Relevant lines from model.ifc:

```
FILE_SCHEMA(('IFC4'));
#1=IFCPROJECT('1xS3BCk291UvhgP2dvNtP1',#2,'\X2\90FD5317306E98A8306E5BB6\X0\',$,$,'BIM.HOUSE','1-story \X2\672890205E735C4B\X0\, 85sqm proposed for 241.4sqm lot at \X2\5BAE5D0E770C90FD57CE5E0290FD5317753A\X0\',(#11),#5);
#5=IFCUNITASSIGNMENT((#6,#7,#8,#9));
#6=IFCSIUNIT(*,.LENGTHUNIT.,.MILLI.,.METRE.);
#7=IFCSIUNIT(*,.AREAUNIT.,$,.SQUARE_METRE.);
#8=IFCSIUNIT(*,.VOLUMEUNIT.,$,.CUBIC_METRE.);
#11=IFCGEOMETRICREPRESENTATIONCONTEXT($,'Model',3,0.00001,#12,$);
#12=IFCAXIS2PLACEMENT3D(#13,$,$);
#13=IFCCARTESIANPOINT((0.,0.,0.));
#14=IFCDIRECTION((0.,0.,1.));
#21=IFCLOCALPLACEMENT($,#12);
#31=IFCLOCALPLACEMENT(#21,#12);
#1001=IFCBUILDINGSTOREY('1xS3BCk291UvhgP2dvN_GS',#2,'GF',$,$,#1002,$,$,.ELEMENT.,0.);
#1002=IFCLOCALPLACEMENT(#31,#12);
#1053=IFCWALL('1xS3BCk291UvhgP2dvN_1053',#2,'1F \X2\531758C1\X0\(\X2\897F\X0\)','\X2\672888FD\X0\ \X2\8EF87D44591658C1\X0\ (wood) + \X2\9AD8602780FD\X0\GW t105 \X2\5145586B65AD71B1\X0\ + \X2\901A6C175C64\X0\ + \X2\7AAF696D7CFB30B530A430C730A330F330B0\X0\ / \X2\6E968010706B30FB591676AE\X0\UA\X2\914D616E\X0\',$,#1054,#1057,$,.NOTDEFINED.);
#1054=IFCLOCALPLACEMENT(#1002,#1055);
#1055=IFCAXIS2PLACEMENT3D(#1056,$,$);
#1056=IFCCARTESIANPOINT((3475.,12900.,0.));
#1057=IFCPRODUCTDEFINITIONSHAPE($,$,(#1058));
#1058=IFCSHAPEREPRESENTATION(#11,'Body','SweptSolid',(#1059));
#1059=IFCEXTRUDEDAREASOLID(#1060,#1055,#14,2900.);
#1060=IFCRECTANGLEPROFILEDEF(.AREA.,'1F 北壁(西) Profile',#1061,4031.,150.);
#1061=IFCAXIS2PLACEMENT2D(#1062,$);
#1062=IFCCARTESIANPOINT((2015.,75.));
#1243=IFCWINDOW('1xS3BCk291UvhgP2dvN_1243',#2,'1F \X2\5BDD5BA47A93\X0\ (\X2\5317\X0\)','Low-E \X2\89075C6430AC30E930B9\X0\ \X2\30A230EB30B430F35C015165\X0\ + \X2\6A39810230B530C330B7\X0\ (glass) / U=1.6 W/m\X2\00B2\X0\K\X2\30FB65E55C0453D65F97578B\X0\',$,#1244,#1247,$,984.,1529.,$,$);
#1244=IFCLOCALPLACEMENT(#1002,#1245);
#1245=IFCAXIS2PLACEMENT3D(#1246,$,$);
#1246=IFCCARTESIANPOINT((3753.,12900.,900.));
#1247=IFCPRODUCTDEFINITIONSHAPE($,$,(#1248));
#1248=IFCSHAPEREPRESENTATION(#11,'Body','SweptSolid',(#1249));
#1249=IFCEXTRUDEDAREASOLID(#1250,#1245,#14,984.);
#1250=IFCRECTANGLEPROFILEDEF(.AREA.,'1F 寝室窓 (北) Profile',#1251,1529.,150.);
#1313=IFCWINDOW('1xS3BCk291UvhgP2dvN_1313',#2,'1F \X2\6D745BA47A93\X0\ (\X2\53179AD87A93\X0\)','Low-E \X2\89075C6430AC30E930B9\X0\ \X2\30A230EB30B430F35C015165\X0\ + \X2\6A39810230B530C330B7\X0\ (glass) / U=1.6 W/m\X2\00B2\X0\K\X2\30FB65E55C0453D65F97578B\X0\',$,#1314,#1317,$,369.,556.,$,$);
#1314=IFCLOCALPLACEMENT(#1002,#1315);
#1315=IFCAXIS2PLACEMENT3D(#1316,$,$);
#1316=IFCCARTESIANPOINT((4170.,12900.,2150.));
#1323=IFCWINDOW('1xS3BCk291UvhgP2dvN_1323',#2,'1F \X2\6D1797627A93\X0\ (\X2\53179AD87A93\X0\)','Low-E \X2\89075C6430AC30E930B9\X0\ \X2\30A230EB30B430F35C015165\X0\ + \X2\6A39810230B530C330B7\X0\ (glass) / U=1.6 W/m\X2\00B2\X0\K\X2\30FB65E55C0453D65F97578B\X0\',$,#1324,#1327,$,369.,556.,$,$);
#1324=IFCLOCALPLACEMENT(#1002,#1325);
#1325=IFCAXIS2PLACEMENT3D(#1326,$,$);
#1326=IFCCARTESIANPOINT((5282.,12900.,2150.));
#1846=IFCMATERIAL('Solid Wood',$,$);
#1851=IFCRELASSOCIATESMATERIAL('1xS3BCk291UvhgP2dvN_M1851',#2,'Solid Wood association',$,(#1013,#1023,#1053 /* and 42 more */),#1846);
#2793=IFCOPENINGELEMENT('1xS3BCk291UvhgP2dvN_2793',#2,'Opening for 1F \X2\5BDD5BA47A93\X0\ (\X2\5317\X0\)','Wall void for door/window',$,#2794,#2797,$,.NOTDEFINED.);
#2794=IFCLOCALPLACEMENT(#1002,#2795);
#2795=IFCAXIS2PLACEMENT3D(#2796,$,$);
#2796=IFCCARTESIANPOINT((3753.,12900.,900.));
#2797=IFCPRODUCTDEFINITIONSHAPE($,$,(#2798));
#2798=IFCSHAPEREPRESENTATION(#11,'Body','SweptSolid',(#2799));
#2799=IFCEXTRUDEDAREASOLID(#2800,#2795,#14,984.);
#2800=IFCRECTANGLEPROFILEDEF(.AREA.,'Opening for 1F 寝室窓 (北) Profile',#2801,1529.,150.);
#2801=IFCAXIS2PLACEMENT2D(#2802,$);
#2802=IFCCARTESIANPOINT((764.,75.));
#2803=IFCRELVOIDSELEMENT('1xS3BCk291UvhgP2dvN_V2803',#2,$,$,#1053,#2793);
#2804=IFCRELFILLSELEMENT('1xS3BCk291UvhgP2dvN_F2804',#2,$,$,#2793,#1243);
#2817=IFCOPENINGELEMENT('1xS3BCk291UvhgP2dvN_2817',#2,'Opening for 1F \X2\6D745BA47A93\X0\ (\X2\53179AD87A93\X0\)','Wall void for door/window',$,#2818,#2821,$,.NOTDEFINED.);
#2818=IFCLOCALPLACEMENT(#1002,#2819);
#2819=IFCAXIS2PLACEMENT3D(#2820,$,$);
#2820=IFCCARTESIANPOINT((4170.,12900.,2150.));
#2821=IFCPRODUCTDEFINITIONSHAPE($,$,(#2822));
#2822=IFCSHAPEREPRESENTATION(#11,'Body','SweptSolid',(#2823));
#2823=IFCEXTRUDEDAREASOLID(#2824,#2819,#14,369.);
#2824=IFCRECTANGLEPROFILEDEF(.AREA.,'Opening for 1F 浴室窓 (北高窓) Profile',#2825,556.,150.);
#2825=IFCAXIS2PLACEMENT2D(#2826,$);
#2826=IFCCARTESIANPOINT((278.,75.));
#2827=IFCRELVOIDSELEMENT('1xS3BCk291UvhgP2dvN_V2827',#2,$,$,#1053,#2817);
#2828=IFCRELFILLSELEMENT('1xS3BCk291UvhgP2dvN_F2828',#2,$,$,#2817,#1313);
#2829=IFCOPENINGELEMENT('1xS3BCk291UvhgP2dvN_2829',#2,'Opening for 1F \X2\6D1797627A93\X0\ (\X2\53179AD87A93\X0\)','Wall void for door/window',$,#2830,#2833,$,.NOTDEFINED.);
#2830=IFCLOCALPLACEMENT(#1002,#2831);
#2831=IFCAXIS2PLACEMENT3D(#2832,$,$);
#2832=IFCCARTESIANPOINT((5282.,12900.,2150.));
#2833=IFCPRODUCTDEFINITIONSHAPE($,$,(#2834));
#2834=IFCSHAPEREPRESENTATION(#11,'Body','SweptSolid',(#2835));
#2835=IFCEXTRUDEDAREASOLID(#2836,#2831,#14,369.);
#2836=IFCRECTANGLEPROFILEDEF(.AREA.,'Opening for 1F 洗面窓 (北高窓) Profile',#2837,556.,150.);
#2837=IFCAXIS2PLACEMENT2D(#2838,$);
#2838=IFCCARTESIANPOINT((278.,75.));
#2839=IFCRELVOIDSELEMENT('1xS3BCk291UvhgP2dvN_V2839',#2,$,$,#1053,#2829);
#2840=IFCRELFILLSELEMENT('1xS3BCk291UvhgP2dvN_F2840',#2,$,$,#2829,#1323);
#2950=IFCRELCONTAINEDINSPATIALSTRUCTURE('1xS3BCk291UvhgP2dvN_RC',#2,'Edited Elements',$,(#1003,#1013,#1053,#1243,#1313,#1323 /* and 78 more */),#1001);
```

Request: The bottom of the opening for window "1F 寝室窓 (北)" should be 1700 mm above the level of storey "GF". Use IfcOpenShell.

```python
import numpy as np
import ifcopenshell
import ifcopenshell.api.geometry
import ifcopenshell.geom
import ifcopenshell.util.element
import ifcopenshell.util.placement
import ifcopenshell.util.shape
import ifcopenshell.util.unit

model = ifcopenshell.open("model.ifc")
unit_scale = ifcopenshell.util.unit.calculate_unit_scale(model)

window = model.by_guid("1xS3BCk291UvhgP2dvN_1243")
opening = window.FillsVoids[0].RelatingOpeningElement
storey = ifcopenshell.util.element.get_container(window, ifc_class="IfcBuildingStorey")
level = ifcopenshell.util.placement.get_local_placement(storey.ObjectPlacement)[2, 3]

# The opening's origin need not be at the sill, so measure its lowest point.
shape = ifcopenshell.geom.create_shape(ifcopenshell.geom.settings(), opening)
bottom = ifcopenshell.util.shape.get_shape_bottom_elevation(shape, shape.geometry) / unit_scale
dz = level + 1.7 / unit_scale - bottom

shift = np.array([0.0, 0.0, dz])
# The window is not placed relative to its opening, so move both.
for product in (opening, window):
    matrix = ifcopenshell.util.placement.get_local_placement(product.ObjectPlacement)
    matrix[:3, 3] += shift
    ifcopenshell.api.geometry.edit_object_placement(model, product=product, matrix=matrix, is_si=False)

print(f"moved by {dz * unit_scale:+.3f} m")

model.write("model_v2.ifc")
```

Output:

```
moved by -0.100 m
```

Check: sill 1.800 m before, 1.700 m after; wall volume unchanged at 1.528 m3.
